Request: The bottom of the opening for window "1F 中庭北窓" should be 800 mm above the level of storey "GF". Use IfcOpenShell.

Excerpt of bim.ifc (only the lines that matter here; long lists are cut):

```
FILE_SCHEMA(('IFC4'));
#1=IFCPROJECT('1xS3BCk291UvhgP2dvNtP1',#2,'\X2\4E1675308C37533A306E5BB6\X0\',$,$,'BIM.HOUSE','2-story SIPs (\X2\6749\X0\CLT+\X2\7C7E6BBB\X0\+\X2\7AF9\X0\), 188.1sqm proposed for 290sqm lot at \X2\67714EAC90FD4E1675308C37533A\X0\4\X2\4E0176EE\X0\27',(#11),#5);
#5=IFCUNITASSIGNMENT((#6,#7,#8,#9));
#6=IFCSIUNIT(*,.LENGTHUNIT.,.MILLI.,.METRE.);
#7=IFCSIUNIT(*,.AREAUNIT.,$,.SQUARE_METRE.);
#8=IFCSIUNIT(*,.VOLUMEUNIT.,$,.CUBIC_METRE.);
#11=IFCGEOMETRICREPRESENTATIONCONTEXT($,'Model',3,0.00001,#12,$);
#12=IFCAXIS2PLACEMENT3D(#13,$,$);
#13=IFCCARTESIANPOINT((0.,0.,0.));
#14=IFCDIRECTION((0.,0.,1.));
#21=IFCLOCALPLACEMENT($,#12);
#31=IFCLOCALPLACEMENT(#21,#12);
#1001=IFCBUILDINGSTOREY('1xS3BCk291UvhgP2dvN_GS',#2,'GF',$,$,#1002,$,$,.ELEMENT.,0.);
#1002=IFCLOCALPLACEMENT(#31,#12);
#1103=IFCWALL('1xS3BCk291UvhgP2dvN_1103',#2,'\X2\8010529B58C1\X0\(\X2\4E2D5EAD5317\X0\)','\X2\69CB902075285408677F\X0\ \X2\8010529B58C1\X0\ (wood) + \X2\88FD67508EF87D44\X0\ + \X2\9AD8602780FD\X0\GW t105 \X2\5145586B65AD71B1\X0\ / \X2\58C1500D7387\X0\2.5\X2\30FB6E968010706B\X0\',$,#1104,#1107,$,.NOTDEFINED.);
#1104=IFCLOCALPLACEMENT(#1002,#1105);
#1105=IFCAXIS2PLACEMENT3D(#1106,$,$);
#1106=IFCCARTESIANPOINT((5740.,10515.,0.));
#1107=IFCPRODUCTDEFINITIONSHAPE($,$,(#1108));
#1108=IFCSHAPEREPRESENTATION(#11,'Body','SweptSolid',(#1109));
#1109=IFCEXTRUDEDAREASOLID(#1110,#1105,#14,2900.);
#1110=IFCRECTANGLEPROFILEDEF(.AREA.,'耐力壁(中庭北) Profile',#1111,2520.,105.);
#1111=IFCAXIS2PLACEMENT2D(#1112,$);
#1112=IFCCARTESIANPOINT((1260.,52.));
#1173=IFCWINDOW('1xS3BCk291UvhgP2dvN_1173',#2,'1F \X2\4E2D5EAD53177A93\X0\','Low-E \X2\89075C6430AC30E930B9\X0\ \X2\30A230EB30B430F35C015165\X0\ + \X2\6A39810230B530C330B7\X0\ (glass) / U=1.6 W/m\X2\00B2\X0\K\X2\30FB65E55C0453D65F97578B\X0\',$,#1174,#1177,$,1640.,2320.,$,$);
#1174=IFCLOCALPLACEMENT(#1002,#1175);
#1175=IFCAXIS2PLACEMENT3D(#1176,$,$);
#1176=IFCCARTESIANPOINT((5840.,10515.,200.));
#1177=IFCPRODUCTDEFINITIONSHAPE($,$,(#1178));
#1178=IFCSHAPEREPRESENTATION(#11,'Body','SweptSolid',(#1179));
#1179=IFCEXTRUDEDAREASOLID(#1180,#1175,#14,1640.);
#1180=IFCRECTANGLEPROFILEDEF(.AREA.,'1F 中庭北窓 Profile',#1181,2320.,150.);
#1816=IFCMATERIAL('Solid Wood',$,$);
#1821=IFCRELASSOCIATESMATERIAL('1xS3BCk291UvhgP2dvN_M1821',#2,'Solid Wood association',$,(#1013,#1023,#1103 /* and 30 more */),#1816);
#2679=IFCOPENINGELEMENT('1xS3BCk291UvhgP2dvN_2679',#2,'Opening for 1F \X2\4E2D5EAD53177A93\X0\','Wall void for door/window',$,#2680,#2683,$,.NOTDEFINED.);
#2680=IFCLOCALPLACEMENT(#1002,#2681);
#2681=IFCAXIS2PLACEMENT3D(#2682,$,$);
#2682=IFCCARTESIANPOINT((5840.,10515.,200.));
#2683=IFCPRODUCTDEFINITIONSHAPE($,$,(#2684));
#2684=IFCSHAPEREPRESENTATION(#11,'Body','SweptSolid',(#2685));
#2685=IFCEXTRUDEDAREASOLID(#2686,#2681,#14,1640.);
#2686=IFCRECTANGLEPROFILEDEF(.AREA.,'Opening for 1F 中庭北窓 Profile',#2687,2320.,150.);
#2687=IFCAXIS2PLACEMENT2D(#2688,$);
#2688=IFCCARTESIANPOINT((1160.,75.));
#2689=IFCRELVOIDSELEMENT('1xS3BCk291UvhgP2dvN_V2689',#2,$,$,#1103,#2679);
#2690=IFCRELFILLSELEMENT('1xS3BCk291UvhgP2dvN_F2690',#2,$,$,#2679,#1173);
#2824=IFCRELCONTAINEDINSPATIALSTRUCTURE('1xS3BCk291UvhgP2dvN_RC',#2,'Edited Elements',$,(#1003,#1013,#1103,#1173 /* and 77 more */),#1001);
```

```python
import numpy as np
import ifcopenshell
import ifcopenshell.api.geometry
import ifcopenshell.geom
import ifcopenshell.util.element
import ifcopenshell.util.placement
import ifcopenshell.util.shape
import ifcopenshell.util.unit

model = ifcopenshell.open("bim.ifc")
unit_scale = ifcopenshell.util.unit.calculate_unit_scale(model)

window = model.by_id(1173)
opening = window.FillsVoids[0].RelatingOpeningElement
storey = ifcopenshell.util.element.get_container(window, ifc_class="IfcBuildingStorey")
level = ifcopenshell.util.placement.get_local_placement(storey.ObjectPlacement)[2, 3]

# The opening's origin need not be at the sill, so measure its lowest point.
shape = ifcopenshell.geom.create_shape(ifcopenshell.geom.settings(), opening)
bottom = ifcopenshell.util.shape.get_shape_bottom_elevation(shape, shape.geometry) / unit_scale
dz = level + 0.8 / unit_scale - bottom

shift = np.array([0.0, 0.0, dz])
# The window is not placed relative to its opening, so move both.
for product in (opening, window):
    matrix = ifcopenshell.util.placement.get_local_placement(product.ObjectPlacement)
    matrix[:3, 3] += shift
    ifcopenshell.api.geometry.edit_object_placement(model, product=product, matrix=matrix, is_si=False)

print(f"moved by {dz * unit_scale:+.3f} m")

model.write("bim_rev.ifc")
```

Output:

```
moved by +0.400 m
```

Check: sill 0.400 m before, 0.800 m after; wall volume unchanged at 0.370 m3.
